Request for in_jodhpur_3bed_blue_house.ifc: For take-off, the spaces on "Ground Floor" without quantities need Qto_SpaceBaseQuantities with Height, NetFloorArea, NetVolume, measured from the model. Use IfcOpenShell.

First a look at what the model holds.

```python
import ifcopenshell
import ifcopenshell.util.element
import ifcopenshell.util.unit

model = ifcopenshell.open("in_jodhpur_3bed_blue_house.ifc")
print(model.schema)
for unit_type in ("LENGTHUNIT", "AREAUNIT", "VOLUMEUNIT"):
    print(unit_type, ifcopenshell.util.unit.calculate_unit_scale(model, unit_type))
storey = next(s for s in model.by_type("IfcBuildingStorey") if s.Name == "Ground Floor")
spaces = [e for e in ifcopenshell.util.element.get_decomposition(storey) if e.is_a("IfcSpace")]
for e in sorted(spaces, key=lambda e: e.id()):
    print(e.id(), e.is_a(), e.Name, list(ifcopenshell.util.element.get_psets(e, qtos_only=True)), sep=" | ")
```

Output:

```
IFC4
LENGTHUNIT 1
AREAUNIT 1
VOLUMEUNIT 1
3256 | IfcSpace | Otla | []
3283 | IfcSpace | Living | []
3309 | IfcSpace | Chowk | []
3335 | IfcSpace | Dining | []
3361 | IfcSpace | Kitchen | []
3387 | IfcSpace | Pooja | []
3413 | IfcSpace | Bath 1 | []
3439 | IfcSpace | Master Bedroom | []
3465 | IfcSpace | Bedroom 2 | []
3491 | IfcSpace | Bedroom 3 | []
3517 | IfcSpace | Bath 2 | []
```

```python
import ifcopenshell
import ifcopenshell.api.pset
import ifcopenshell.geom
import ifcopenshell.util.element
import ifcopenshell.util.shape
import ifcopenshell.util.unit

model = ifcopenshell.open("in_jodhpur_3bed_blue_house.ifc")
unit_scale = ifcopenshell.util.unit.calculate_unit_scale(model)
area_scale = ifcopenshell.util.unit.calculate_unit_scale(model, "AREAUNIT")
volume_scale = ifcopenshell.util.unit.calculate_unit_scale(model, "VOLUMEUNIT")
settings = ifcopenshell.geom.settings()

storey = next(s for s in model.by_type("IfcBuildingStorey") if s.Name == "Ground Floor")
spaces = [e for e in ifcopenshell.util.element.get_decomposition(storey) if e.is_a("IfcSpace")]

for e in sorted(spaces, key=lambda e: e.id()):
    if ifcopenshell.util.element.get_psets(e, qtos_only=True, should_inherit=False):
        continue
    # Geometry comes back in metres, in the element's own axes.
    shape = ifcopenshell.geom.create_shape(settings, e)
    values = {
        "Height": ifcopenshell.util.shape.get_z(shape.geometry) / unit_scale,
        "NetFloorArea": ifcopenshell.util.shape.get_footprint_area(shape.geometry) / area_scale,
        "NetVolume": ifcopenshell.util.shape.get_volume(shape.geometry) / volume_scale,
    }
    qto = ifcopenshell.api.pset.add_qto(model, product=e, name="Qto_SpaceBaseQuantities")
    ifcopenshell.api.pset.edit_qto(model, qto=qto, properties=values)
    print(e.id(), {k: round(v, 3) for k, v in values.items()})

model.write("in_jodhpur_3bed_blue_house_rev.ifc")
```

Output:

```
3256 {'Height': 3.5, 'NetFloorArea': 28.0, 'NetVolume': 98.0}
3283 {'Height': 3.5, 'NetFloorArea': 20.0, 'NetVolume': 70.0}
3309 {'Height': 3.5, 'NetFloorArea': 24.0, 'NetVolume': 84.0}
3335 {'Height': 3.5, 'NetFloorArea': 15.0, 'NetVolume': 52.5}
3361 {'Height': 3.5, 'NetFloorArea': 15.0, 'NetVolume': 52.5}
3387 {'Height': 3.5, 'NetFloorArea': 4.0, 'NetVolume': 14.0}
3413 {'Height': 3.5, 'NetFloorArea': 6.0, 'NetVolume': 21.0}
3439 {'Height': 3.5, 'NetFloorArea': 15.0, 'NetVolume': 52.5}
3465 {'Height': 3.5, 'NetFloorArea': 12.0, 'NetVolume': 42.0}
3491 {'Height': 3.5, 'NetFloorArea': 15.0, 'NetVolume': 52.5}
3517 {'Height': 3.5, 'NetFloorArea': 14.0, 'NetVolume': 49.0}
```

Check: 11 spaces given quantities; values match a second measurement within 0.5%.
